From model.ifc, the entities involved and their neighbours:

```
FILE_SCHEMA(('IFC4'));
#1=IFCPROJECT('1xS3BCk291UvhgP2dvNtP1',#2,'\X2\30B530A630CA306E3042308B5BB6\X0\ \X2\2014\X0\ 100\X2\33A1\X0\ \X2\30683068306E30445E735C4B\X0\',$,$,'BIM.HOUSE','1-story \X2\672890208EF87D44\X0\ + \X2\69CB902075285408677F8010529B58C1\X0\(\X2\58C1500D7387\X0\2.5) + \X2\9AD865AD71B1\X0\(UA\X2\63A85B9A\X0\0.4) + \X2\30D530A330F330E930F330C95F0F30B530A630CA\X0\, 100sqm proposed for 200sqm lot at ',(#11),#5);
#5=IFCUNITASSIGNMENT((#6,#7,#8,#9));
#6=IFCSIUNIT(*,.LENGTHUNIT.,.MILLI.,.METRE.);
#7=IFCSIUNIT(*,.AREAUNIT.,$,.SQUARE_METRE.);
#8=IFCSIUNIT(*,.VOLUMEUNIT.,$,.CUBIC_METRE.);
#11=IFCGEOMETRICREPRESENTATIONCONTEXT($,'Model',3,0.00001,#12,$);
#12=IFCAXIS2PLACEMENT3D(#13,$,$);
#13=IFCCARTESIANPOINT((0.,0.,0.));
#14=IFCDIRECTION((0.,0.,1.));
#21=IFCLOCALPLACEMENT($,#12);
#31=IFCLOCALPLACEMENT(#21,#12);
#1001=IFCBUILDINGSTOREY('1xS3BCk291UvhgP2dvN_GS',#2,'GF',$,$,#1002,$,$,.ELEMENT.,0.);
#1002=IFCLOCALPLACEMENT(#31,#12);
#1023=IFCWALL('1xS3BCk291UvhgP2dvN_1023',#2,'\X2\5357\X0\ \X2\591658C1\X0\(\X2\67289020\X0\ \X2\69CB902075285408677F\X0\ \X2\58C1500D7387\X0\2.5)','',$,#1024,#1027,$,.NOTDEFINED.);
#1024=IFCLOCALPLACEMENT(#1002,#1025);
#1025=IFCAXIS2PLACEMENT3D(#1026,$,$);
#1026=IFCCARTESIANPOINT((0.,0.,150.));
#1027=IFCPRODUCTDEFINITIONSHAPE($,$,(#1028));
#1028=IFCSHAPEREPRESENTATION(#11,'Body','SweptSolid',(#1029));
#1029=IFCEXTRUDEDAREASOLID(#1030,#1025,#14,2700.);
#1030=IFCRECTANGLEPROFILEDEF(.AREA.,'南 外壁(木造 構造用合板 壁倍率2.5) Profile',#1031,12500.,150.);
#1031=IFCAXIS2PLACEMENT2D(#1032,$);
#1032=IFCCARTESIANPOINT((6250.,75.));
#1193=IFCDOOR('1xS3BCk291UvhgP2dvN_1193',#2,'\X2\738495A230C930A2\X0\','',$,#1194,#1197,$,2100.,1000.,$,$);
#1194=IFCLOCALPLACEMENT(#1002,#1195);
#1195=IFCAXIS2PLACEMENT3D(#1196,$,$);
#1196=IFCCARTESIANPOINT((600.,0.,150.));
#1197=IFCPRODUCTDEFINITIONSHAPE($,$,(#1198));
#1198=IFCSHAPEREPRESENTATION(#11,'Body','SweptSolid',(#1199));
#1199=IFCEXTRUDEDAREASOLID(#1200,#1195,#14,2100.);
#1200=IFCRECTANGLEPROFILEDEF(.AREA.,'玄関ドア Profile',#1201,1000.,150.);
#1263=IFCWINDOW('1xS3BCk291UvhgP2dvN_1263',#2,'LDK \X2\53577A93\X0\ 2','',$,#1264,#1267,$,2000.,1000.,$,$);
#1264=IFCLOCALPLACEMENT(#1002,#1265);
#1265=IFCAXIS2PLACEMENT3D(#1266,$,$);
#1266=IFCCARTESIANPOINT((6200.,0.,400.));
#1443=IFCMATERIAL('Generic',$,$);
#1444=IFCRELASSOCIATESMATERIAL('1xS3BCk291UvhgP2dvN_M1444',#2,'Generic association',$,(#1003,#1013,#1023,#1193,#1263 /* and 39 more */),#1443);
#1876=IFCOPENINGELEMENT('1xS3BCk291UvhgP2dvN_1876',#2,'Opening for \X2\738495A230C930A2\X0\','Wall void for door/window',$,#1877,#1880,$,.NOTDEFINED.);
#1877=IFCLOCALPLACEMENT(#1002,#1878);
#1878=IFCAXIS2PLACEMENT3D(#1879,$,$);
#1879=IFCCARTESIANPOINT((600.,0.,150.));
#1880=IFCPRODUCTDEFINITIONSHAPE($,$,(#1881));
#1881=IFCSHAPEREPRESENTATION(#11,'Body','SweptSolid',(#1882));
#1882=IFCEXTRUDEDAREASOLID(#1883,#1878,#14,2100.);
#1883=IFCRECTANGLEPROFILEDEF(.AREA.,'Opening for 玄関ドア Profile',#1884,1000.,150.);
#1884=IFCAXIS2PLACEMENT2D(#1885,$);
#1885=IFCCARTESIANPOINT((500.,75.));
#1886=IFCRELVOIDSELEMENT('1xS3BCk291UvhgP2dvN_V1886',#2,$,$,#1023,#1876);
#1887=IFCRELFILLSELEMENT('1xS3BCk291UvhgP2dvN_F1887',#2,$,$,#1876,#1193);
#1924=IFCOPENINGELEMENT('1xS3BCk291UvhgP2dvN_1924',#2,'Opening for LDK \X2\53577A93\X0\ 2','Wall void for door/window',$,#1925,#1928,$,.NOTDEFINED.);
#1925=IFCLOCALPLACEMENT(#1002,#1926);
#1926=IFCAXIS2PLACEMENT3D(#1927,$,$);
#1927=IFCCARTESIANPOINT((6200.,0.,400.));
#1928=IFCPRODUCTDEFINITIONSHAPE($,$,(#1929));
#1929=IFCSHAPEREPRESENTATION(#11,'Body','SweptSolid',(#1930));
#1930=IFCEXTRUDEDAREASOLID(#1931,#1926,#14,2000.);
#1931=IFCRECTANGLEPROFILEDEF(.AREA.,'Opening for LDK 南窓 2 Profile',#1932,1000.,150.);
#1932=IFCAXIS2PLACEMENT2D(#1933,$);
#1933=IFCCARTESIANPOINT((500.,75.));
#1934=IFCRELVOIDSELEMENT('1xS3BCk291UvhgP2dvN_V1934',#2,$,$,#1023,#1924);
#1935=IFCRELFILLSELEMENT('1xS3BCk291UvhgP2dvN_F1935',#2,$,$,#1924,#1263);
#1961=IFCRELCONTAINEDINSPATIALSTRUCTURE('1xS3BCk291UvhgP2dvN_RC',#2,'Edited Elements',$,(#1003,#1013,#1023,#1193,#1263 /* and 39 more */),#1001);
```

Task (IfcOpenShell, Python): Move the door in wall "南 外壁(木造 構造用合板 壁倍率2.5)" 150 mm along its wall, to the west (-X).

```python
import ifcopenshell
import ifcopenshell.api.geometry
import ifcopenshell.util.placement

model = ifcopenshell.open("model.ifc")

door = model.by_id(1193)
opening = door.FillsVoids[0].RelatingOpeningElement
wall = opening.VoidsElements[0].RelatingBuildingElement

wall_matrix = ifcopenshell.util.placement.get_local_placement(wall.ObjectPlacement)
shift = wall_matrix[:3, 0] * -150.0
before = ifcopenshell.util.placement.get_local_placement(door.ObjectPlacement)[:3, 3].copy()

# The door is not placed relative to its opening, so move both.
for product in (opening, door):
    matrix = ifcopenshell.util.placement.get_local_placement(product.ObjectPlacement)
    matrix[:3, 3] += shift
    ifcopenshell.api.geometry.edit_object_placement(model, product=product, matrix=matrix, is_si=False)

after = ifcopenshell.util.placement.get_local_placement(door.ObjectPlacement)[:3, 3]
print("door moved by", (after - before).round(3) + 0.0)

model.write("model_updated.ifc")
```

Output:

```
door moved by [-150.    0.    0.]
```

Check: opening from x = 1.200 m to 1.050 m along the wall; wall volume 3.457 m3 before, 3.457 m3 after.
